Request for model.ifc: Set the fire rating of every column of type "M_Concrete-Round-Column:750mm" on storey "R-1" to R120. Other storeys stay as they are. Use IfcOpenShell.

First a look at what the model holds.

```python
import ifcopenshell
import ifcopenshell.util.element

model = ifcopenshell.open("model.ifc")
print(model.schema)
storey = next(s for s in model.by_type("IfcBuildingStorey") if s.Name == "R-1")
columns = [e for e in ifcopenshell.util.element.get_decomposition(storey) if e.is_a("IfcColumn")]
seen = {}
for e in columns:
    element_type = ifcopenshell.util.element.get_type(e)
    key = (element_type.Name if element_type != e and element_type else None, ifcopenshell.util.element.get_pset(e, "Pset_ColumnCommon", "FireRating"))
    seen[key] = seen.get(key, 0) + 1
for (name, value), count in sorted(seen.items(), key=str):
    print(count, "x", name, "|", value)
```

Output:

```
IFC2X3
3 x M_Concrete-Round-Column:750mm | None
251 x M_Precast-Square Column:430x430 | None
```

```python
import ifcopenshell
import ifcopenshell.api.pset
import ifcopenshell.util.element

model = ifcopenshell.open("model.ifc")

storey = next(s for s in model.by_type("IfcBuildingStorey") if s.Name == "R-1")
columns = [e for e in ifcopenshell.util.element.get_decomposition(storey) if e.is_a("IfcColumn")]

count = 0
for e in columns:
    element_type = ifcopenshell.util.element.get_type(e)
    if element_type in (None, e) or element_type.Name != "M_Concrete-Round-Column:750mm":
        continue
    # add_pset returns the element's existing set when there is one.
    pset = ifcopenshell.api.pset.add_pset(model, product=e, name="Pset_ColumnCommon")
    ifcopenshell.api.pset.edit_pset(model, pset=pset, properties={"FireRating": "R120"})
    count += 1

print(count, "columns updated")

model.write("model_edited.ifc")
```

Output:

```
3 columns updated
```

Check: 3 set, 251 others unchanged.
